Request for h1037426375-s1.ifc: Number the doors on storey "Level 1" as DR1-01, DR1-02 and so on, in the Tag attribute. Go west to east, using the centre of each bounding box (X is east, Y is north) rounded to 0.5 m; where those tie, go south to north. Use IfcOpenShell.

First a look at what the model holds.

```python
import ifcopenshell
import ifcopenshell.util.element
import ifcopenshell.util.placement

model = ifcopenshell.open("h1037426375-s1.ifc")
print(model.schema)
storey = next(s for s in model.by_type("IfcBuildingStorey") if s.Name == "Level 1")
doors = [e for e in ifcopenshell.util.element.get_decomposition(storey) if e.is_a("IfcDoor")]
for e in sorted(doors, key=lambda e: e.id()):
    origin = ifcopenshell.util.placement.get_local_placement(e.ObjectPlacement)[:3, 3]
    print(e.id(), e.Tag, e.Name, origin.round(2) + 0.0, sep=" | ")
```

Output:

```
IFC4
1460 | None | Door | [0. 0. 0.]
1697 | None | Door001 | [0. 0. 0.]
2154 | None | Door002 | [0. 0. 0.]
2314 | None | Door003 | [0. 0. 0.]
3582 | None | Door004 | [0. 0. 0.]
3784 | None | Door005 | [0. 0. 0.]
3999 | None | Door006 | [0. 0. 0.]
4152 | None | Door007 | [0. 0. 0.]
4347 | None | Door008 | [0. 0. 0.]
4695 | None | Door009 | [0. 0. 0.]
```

```python
import ifcopenshell
import ifcopenshell.geom
import ifcopenshell.util.element
import ifcopenshell.util.shape

model = ifcopenshell.open("h1037426375-s1.ifc")
settings = ifcopenshell.geom.settings()
settings.set("use-world-coords", True)


def centre(element):
    shape = ifcopenshell.geom.create_shape(settings, element)
    return ifcopenshell.util.shape.get_bbox_centroid(shape.geometry)


storey = next(s for s in model.by_type("IfcBuildingStorey") if s.Name == "Level 1")
doors = [e for e in ifcopenshell.util.element.get_decomposition(storey) if e.is_a("IfcDoor")]

# Insertion points can sit at a corner or the storey origin, so sort by the geometry (in metres).
centres = {e: centre(e) for e in doors}
doors.sort(key=lambda e: (round(centres[e][0] / 0.5), centres[e][1]))

for i, e in enumerate(doors, start=1):
    number = f"DR1-{i:02d}"
    e.Tag = number
    print(e.id(), number)

model.write("h1037426375-s1_v2.ifc")
```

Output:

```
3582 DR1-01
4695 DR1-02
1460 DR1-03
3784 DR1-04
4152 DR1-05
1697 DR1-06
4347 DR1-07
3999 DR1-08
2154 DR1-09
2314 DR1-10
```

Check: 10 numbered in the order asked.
